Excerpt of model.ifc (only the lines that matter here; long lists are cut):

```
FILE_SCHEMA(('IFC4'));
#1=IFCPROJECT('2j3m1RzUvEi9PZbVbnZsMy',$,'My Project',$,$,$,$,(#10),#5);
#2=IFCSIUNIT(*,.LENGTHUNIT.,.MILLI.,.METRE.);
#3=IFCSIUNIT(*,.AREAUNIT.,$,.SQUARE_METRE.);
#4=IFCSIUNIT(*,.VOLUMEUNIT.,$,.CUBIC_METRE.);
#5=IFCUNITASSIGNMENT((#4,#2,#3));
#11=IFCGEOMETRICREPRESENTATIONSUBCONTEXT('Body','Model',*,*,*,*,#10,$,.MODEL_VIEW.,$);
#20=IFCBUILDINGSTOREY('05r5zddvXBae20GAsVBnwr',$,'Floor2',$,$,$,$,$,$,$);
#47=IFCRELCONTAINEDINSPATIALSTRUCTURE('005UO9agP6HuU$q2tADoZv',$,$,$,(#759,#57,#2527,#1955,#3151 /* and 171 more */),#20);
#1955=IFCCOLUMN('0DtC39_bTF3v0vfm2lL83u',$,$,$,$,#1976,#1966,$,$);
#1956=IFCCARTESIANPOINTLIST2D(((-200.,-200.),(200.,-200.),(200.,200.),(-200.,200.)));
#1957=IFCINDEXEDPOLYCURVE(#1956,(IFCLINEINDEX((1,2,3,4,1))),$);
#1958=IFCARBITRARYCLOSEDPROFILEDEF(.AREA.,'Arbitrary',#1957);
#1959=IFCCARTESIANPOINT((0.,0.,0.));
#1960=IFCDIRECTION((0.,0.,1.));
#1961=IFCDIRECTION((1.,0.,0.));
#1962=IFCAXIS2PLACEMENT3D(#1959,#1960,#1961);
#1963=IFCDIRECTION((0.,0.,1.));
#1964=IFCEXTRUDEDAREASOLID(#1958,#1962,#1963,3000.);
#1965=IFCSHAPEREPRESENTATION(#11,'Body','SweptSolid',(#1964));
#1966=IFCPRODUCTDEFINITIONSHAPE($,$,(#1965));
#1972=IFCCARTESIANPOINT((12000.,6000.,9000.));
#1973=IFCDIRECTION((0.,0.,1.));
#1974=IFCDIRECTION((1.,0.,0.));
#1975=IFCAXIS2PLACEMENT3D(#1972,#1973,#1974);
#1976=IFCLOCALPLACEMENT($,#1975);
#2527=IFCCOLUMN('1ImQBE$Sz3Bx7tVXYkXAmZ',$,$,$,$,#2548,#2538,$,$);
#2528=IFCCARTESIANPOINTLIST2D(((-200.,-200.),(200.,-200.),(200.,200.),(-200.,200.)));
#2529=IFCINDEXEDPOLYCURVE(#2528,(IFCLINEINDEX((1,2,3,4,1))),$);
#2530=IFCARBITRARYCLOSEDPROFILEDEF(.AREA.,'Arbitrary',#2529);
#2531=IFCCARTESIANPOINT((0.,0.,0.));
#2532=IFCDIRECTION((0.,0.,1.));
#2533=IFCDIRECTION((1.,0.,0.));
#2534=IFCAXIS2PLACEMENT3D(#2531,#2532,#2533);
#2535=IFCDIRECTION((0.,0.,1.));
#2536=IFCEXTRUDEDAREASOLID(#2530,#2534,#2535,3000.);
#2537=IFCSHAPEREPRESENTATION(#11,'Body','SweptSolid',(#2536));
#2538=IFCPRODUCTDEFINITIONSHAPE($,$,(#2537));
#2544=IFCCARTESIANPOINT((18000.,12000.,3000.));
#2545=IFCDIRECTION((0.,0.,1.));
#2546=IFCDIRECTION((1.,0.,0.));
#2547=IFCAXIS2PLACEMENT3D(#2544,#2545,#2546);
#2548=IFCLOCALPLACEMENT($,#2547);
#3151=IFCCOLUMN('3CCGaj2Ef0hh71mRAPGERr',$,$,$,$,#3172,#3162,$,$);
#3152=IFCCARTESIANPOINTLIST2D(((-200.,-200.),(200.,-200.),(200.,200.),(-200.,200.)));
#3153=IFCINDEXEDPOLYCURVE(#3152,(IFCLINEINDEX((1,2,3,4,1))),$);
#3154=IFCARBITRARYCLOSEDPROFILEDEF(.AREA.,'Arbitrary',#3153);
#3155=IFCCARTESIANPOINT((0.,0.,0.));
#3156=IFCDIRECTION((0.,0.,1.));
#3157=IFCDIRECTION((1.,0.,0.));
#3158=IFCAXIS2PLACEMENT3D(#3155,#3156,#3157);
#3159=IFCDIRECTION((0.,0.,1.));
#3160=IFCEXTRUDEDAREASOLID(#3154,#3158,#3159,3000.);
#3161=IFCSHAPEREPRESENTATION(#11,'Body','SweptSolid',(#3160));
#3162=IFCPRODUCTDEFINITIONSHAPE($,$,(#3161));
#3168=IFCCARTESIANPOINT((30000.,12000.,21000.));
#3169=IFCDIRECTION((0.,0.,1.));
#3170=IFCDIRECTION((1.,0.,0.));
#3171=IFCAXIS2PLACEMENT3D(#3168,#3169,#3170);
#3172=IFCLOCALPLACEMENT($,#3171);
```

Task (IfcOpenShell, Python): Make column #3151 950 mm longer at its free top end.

```python
import ifcopenshell
import ifcopenshell.util.representation

model = ifcopenshell.open("model.ifc")

member = model.by_guid("3CCGaj2Ef0hh71mRAPGERr")
change = 950.0

# The extrusion runs towards the end named, so only its depth changes.
body = ifcopenshell.util.representation.get_representation(member, "Model", "Body")
solid = body.Items[0]
old_length = solid.Depth
solid.Depth += change

print(f"length {old_length:g} -> {solid.Depth:g}")

model.write("model_edited.ifc")
```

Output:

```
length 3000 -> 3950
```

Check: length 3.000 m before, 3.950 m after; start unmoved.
